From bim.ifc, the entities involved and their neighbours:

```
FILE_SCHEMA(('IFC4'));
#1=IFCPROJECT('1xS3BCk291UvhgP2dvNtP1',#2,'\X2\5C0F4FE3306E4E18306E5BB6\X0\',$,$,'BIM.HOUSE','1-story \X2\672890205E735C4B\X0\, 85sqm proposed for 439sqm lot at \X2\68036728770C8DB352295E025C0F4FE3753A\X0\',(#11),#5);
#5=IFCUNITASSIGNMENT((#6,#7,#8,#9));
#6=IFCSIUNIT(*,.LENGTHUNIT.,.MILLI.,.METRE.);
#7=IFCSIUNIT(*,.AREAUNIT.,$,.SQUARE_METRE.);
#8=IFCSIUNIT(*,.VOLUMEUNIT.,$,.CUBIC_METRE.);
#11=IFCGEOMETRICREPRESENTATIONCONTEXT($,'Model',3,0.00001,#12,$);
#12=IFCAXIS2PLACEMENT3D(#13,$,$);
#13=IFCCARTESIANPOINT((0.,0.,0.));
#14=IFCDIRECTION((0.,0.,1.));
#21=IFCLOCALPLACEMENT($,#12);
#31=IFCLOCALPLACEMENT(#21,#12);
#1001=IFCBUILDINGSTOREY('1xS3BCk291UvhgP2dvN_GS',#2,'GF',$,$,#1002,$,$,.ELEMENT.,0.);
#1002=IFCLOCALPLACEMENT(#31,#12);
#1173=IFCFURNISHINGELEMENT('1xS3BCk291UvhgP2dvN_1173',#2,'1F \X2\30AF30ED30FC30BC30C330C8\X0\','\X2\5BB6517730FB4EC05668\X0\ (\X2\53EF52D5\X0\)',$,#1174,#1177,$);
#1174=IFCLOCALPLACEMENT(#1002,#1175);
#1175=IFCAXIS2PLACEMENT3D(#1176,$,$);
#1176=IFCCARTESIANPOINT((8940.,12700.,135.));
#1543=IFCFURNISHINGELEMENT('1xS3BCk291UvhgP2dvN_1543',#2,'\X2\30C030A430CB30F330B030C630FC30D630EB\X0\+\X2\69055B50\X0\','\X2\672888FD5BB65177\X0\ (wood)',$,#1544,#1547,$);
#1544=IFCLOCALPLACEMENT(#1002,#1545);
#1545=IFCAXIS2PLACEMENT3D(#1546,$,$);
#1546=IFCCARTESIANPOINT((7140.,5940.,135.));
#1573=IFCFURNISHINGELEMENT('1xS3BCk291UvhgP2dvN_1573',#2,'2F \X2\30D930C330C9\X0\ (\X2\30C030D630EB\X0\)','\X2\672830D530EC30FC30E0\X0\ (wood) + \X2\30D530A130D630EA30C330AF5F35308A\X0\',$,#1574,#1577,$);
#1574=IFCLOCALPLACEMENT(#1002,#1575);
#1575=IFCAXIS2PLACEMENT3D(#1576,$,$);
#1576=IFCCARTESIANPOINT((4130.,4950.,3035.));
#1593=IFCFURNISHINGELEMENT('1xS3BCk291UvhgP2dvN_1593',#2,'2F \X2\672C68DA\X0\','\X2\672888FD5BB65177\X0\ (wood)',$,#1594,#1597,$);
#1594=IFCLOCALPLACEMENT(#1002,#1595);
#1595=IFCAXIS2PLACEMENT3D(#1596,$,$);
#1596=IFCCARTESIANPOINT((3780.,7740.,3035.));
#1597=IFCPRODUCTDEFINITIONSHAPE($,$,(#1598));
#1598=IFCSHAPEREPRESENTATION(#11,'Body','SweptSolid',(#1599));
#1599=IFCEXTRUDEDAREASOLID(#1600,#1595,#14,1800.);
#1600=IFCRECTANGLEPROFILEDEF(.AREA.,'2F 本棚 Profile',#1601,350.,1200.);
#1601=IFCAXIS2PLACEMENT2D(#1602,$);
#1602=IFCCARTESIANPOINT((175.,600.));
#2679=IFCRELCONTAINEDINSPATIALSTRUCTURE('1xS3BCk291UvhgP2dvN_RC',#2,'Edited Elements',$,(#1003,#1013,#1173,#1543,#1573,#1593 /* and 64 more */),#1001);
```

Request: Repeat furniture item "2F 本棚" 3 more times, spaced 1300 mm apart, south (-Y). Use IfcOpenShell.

```python
import numpy as np
import ifcopenshell
import ifcopenshell.api.geometry
import ifcopenshell.api.root
import ifcopenshell.util.element
import ifcopenshell.util.placement
import ifcopenshell.util.unit

model = ifcopenshell.open("bim.ifc")
unit_scale = ifcopenshell.util.unit.calculate_unit_scale(model)


def reuse_history(source, copy):
    """copy_class also copies each property set's owner history, people and application; keep the originals."""
    for rel in copy.IsDefinedBy:
        if rel.is_a("IfcRelDefinesByProperties") and (history := rel.RelatingPropertyDefinition.OwnerHistory):
            rel.RelatingPropertyDefinition.OwnerHistory = source.OwnerHistory
            ifcopenshell.util.element.remove_deep2(model, history)


source = model.by_id(1593)
base = ifcopenshell.util.placement.get_local_placement(source.ObjectPlacement)
step = np.array([0.0, -1.0, 0.0]) * 1.3 / unit_scale

for i in range(1, 4):
    copy = ifcopenshell.api.root.copy_class(model, product=source)
    copy.Representation = ifcopenshell.util.element.copy_deep(
        model, source.Representation, exclude=["IfcGeometricRepresentationContext", "IfcRepresentationMap"]
    )
    reuse_history(source, copy)
    matrix = base.copy()
    matrix[:3, 3] += i * step
    print("added at", matrix[:3, 3].round(3) + 0.0)
    ifcopenshell.api.geometry.edit_object_placement(model, product=copy, matrix=matrix, is_si=False)

model.write("bim_updated.ifc")
```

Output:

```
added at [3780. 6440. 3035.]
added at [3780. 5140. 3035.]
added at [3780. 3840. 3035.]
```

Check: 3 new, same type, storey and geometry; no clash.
